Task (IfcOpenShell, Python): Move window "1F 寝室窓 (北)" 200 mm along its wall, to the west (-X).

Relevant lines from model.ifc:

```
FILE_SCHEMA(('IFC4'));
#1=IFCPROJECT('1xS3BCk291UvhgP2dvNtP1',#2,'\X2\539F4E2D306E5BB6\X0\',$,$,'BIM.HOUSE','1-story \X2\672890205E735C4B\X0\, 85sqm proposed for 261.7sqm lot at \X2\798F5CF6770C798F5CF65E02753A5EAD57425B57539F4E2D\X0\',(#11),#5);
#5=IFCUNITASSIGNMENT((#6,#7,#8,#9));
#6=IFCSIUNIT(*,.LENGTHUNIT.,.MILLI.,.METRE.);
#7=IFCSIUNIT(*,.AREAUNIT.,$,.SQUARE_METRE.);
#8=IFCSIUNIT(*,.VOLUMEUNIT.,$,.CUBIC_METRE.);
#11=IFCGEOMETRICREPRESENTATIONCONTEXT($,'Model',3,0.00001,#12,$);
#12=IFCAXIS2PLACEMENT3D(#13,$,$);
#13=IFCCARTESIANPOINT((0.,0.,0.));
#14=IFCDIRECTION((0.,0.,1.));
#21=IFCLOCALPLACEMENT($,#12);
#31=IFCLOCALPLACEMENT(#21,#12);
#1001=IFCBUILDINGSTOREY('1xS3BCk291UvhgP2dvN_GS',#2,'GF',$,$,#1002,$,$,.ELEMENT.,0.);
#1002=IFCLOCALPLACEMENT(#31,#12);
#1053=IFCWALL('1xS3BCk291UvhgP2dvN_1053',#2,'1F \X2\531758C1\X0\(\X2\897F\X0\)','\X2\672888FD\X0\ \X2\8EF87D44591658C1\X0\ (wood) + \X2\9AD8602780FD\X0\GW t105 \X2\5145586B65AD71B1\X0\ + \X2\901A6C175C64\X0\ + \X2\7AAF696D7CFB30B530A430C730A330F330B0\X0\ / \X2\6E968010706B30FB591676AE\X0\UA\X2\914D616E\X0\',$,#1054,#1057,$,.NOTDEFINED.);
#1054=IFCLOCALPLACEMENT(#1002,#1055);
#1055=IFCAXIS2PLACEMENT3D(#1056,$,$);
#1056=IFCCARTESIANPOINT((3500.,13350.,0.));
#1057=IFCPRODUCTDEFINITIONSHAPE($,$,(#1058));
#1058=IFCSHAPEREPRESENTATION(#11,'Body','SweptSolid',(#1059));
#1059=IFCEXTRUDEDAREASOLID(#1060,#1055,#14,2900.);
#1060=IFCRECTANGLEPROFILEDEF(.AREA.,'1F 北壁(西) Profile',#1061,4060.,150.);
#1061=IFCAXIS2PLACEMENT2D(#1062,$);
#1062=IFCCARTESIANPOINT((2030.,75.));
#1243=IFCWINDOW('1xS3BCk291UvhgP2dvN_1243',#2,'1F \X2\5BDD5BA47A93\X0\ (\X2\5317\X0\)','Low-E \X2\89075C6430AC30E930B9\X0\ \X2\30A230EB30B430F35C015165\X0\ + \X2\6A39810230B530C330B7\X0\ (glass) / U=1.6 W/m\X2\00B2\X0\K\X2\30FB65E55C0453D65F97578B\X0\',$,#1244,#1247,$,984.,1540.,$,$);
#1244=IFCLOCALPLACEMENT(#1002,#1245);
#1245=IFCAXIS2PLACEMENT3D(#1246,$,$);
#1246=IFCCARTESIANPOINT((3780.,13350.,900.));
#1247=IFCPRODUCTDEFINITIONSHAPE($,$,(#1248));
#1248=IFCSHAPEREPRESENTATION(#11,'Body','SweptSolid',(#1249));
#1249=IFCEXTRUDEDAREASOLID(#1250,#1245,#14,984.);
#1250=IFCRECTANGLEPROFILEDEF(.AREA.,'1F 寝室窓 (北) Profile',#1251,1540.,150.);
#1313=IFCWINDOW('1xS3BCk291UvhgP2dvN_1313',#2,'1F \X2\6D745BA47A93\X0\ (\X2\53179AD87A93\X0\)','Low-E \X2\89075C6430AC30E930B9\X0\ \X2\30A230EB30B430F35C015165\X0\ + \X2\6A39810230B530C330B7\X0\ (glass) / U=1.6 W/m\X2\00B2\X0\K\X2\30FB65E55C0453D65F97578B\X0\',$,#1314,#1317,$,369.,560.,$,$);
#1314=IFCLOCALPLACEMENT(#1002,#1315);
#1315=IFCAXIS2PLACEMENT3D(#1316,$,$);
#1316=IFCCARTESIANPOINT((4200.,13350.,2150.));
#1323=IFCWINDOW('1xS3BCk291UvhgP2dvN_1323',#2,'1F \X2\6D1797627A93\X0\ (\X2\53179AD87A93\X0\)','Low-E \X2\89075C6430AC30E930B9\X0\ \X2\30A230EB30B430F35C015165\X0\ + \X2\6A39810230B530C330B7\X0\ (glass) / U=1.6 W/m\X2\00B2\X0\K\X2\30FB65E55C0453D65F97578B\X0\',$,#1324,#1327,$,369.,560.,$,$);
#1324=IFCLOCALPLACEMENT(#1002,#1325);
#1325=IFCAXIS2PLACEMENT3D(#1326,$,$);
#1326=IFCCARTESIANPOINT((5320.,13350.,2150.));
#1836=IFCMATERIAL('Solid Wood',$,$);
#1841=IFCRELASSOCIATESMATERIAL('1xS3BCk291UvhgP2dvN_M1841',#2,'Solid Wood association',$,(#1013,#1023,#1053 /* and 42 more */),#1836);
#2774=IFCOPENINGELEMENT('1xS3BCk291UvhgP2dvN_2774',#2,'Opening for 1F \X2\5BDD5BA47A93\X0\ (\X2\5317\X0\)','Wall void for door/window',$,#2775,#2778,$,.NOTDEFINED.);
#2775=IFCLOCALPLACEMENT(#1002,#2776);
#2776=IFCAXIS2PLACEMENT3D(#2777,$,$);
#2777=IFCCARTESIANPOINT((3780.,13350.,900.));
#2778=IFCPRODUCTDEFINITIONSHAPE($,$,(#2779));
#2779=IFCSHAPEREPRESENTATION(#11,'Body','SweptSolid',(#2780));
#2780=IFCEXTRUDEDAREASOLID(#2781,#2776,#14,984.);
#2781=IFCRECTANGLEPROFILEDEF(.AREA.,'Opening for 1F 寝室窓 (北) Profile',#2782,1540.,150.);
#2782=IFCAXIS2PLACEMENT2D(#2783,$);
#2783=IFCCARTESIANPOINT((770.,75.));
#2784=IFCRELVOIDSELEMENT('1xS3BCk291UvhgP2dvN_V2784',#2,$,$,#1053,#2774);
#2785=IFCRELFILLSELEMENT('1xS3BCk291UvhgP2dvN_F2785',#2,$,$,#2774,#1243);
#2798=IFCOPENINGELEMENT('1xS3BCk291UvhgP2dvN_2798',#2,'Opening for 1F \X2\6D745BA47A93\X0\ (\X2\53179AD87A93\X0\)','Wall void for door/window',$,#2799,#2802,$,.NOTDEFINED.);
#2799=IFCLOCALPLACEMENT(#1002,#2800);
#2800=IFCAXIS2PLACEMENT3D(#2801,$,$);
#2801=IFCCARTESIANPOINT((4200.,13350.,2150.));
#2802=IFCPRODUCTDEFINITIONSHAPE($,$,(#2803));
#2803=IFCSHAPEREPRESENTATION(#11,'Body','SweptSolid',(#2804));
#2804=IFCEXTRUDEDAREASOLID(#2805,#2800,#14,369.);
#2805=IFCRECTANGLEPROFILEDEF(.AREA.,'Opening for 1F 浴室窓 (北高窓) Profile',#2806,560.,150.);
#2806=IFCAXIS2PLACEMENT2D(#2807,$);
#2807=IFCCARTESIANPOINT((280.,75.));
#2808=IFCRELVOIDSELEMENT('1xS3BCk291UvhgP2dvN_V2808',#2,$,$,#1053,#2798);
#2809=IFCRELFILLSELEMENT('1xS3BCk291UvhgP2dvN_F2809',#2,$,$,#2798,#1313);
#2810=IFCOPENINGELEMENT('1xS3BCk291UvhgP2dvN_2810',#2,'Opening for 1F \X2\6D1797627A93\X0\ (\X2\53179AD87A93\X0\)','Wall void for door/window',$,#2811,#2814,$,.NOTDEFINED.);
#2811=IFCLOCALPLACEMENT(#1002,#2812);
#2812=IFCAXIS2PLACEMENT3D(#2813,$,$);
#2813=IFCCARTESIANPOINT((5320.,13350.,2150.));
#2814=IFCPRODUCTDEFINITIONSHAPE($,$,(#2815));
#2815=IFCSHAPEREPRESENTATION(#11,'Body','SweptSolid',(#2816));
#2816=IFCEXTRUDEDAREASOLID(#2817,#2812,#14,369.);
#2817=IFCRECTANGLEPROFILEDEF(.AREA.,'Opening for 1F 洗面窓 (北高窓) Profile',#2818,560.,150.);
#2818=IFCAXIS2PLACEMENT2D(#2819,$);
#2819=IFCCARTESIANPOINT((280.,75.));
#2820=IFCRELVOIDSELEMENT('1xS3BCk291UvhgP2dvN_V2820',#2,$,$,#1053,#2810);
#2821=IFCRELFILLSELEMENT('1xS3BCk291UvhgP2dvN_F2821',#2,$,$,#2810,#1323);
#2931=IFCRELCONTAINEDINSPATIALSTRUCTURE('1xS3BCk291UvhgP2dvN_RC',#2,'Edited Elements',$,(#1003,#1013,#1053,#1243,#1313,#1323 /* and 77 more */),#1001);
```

```python
import ifcopenshell
import ifcopenshell.api.geometry
import ifcopenshell.util.placement
import ifcopenshell.util.unit

model = ifcopenshell.open("model.ifc")
unit_scale = ifcopenshell.util.unit.calculate_unit_scale(model)

window = model.by_guid("1xS3BCk291UvhgP2dvN_1243")
opening = window.FillsVoids[0].RelatingOpeningElement
wall = opening.VoidsElements[0].RelatingBuildingElement

wall_matrix = ifcopenshell.util.placement.get_local_placement(wall.ObjectPlacement)
shift = wall_matrix[:3, 0] * -0.2 / unit_scale
before = ifcopenshell.util.placement.get_local_placement(window.ObjectPlacement)[:3, 3].copy()

# The window is not placed relative to its opening, so move both.
for product in (opening, window):
    matrix = ifcopenshell.util.placement.get_local_placement(product.ObjectPlacement)
    matrix[:3, 3] += shift
    ifcopenshell.api.geometry.edit_object_placement(model, product=product, matrix=matrix, is_si=False)

after = ifcopenshell.util.placement.get_local_placement(window.ObjectPlacement)[:3, 3]
print("window moved by", (after - before).round(3) + 0.0)

model.write("model_edited.ifc")
```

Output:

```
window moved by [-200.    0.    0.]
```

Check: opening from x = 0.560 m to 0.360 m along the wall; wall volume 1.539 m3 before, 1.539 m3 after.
